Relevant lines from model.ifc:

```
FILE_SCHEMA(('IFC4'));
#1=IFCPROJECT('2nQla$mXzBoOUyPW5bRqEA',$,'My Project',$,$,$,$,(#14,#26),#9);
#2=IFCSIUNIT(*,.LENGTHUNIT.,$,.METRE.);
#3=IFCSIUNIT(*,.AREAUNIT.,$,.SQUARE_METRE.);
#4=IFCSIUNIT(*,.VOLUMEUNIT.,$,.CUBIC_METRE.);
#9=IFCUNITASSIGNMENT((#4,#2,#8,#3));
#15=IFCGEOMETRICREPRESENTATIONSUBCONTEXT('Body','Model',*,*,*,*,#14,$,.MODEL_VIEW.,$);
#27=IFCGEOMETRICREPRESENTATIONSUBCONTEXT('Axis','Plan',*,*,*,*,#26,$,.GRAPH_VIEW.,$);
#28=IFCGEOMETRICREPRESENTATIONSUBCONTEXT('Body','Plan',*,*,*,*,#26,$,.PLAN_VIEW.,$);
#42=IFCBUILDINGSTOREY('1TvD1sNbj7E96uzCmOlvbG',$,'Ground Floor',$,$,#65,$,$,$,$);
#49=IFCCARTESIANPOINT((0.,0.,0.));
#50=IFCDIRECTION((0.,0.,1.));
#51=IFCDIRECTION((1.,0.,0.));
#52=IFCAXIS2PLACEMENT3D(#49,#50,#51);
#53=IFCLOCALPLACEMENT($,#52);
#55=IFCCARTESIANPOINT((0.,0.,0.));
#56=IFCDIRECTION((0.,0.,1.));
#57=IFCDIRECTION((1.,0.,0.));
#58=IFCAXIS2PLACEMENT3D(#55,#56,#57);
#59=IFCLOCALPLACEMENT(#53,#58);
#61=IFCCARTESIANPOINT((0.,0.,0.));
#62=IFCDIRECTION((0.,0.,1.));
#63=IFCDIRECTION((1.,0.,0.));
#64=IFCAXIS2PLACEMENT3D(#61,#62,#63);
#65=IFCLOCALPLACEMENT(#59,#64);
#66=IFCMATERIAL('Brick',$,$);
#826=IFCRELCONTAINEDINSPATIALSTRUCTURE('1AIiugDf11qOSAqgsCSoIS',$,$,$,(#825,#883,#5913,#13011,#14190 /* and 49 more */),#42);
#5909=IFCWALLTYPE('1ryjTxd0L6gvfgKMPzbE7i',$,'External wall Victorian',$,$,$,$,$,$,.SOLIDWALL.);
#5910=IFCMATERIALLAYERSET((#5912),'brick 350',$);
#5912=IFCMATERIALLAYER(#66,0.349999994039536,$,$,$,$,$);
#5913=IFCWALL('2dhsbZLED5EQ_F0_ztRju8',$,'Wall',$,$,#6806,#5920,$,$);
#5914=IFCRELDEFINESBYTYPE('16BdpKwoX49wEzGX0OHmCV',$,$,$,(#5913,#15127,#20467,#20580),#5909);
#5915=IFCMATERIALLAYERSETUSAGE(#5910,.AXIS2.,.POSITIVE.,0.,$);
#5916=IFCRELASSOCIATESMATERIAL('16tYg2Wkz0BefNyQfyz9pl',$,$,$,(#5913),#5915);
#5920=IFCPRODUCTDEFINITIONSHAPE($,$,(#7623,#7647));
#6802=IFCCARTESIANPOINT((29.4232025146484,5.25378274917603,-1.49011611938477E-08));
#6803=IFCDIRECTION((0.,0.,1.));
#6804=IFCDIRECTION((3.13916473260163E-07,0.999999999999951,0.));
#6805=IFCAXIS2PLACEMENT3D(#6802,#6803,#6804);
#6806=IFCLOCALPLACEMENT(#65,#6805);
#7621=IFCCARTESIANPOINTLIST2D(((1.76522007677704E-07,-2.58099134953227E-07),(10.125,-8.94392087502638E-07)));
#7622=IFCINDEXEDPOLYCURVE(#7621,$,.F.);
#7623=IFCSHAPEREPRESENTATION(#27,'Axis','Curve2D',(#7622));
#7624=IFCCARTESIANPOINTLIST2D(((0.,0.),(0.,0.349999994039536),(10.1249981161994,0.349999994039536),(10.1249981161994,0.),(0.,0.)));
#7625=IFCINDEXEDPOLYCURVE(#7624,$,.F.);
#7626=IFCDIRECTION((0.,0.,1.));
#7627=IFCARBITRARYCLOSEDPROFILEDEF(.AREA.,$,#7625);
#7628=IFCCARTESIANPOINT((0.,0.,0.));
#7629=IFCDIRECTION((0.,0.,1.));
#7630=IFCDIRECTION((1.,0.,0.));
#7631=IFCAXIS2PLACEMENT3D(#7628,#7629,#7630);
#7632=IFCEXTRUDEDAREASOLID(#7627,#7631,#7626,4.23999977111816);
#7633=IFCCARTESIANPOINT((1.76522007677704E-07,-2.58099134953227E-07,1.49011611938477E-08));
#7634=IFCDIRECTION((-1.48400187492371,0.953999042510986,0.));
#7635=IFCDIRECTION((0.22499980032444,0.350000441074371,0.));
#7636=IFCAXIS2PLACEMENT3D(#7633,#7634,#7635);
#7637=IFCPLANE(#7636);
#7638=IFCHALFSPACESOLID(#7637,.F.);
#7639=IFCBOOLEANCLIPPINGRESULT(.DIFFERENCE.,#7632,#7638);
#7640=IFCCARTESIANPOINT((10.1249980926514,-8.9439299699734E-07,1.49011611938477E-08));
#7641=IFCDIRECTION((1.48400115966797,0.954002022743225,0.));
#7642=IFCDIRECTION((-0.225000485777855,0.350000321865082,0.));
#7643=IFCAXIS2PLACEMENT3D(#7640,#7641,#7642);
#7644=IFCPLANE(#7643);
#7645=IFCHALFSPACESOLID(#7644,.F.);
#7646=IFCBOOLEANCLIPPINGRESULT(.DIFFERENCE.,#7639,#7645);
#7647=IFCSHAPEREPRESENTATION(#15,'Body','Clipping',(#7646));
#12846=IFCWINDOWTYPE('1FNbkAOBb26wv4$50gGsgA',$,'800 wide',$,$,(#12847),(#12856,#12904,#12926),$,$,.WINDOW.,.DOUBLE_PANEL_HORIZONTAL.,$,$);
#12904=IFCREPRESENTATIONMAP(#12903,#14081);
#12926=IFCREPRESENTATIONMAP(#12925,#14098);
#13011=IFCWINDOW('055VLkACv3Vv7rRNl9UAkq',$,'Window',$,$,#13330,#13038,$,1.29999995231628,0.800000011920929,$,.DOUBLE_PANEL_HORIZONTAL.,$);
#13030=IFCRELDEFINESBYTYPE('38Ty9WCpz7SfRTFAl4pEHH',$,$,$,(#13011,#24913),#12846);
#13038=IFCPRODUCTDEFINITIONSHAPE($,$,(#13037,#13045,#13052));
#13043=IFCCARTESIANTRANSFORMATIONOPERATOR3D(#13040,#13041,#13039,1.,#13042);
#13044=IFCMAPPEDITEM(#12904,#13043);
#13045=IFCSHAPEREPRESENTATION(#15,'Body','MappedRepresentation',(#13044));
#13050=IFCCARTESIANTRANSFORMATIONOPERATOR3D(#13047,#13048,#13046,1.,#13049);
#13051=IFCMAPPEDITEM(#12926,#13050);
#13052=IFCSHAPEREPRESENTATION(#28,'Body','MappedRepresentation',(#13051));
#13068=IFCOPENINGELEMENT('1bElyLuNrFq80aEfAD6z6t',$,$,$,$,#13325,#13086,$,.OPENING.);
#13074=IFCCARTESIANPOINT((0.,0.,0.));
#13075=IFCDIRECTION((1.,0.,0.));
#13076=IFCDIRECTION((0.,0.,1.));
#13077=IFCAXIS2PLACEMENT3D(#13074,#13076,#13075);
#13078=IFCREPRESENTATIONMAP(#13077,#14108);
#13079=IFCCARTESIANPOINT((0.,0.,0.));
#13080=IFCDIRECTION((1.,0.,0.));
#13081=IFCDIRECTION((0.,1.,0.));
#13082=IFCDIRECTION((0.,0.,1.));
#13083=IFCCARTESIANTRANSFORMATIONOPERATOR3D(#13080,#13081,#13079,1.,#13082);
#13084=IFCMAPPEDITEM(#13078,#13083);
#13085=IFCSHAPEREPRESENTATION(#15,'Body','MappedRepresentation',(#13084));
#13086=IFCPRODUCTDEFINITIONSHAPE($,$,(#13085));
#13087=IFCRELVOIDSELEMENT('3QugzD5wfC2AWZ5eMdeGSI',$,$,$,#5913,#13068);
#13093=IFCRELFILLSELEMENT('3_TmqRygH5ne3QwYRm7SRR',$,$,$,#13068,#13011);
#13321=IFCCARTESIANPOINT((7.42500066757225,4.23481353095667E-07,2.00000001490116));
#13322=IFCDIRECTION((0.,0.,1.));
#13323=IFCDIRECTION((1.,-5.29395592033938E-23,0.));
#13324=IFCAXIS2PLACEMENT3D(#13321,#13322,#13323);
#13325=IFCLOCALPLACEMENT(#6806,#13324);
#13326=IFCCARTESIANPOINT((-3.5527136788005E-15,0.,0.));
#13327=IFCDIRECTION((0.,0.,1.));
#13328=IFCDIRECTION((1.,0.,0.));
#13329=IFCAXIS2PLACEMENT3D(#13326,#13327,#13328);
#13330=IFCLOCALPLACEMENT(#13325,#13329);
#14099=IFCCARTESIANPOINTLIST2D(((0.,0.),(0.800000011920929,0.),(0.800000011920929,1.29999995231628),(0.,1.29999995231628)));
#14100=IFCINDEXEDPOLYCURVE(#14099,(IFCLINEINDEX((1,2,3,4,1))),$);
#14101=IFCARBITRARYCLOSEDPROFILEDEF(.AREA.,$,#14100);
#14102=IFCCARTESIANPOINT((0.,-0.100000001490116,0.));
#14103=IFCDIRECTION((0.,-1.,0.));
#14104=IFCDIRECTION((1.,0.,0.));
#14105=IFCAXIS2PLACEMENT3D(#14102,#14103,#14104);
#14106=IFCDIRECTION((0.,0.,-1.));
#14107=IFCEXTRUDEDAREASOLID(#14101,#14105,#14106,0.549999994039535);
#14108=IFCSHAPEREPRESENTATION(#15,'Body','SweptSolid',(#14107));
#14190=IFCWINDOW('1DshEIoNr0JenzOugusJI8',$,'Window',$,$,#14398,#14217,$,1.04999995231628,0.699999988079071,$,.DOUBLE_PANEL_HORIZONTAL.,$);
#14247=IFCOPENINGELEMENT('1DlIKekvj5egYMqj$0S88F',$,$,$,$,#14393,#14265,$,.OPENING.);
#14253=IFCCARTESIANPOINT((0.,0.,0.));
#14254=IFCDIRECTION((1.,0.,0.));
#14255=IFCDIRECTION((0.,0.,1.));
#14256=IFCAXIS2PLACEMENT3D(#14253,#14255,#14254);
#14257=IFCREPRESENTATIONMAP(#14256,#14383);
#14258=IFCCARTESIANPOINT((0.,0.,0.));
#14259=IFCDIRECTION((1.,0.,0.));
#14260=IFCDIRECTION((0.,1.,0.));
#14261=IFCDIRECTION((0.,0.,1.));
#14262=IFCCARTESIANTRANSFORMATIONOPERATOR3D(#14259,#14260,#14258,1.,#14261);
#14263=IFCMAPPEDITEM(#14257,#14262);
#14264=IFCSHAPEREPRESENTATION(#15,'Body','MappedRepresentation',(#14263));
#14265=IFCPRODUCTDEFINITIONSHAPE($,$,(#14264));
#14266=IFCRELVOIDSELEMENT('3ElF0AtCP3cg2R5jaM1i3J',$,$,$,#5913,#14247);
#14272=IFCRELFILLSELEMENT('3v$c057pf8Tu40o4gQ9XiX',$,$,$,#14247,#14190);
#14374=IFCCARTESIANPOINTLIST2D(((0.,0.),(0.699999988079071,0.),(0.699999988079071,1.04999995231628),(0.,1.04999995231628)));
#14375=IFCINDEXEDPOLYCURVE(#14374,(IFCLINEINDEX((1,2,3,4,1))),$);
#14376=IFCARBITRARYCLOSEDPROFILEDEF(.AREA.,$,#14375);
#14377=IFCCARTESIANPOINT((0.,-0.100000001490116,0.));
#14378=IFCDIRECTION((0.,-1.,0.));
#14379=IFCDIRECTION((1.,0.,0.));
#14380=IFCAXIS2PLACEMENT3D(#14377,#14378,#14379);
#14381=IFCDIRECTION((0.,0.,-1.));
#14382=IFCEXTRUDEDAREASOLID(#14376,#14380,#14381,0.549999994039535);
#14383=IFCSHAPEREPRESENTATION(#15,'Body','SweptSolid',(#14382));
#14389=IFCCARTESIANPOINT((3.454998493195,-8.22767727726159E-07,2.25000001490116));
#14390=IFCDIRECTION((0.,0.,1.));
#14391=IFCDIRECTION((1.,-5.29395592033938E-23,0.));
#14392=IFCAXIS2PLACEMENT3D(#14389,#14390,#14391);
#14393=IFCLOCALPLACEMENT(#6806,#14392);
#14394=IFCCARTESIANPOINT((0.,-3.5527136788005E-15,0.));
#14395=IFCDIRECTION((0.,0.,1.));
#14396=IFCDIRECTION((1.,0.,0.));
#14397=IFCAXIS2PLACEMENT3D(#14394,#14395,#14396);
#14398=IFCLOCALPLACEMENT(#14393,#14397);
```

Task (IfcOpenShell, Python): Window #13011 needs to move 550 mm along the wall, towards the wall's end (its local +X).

```python
import ifcopenshell
import ifcopenshell.api.geometry
import ifcopenshell.util.placement
import ifcopenshell.util.unit

model = ifcopenshell.open("model.ifc")
unit_scale = ifcopenshell.util.unit.calculate_unit_scale(model)

window = model.by_guid("055VLkACv3Vv7rRNl9UAkq")
opening = window.FillsVoids[0].RelatingOpeningElement
wall = opening.VoidsElements[0].RelatingBuildingElement

wall_matrix = ifcopenshell.util.placement.get_local_placement(wall.ObjectPlacement)
shift = wall_matrix[:3, 0] * 0.55 / unit_scale
before = ifcopenshell.util.placement.get_local_placement(window.ObjectPlacement)[:3, 3].copy()

# The window is placed relative to its opening, so it follows when the opening moves.
matrix = ifcopenshell.util.placement.get_local_placement(opening.ObjectPlacement)
matrix[:3, 3] += shift
ifcopenshell.api.geometry.edit_object_placement(
    model, product=opening, matrix=matrix, is_si=False, should_transform_children=True
)

after = ifcopenshell.util.placement.get_local_placement(window.ObjectPlacement)[:3, 3]
print("window moved by", (after - before).round(3) + 0.0)

model.write("model_v2.ifc")
```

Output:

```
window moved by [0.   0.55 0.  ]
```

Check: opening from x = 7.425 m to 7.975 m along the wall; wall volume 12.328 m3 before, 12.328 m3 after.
